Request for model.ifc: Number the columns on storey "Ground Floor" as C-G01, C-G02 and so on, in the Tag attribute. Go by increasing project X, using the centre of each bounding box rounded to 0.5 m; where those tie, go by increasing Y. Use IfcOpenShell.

First a look at what the model holds.

```python
import ifcopenshell
import ifcopenshell.util.element
import ifcopenshell.util.placement

model = ifcopenshell.open("model.ifc")
print(model.schema)
storey = next(s for s in model.by_type("IfcBuildingStorey") if s.Name == "Ground Floor")
columns = [e for e in ifcopenshell.util.element.get_decomposition(storey) if e.is_a("IfcColumn")]
for e in sorted(columns, key=lambda e: e.id()):
    origin = ifcopenshell.util.placement.get_local_placement(e.ObjectPlacement)[:3, 3]
    print(e.id(), e.Tag, e.Name, origin.round(2) + 0.0, sep=" | ")
```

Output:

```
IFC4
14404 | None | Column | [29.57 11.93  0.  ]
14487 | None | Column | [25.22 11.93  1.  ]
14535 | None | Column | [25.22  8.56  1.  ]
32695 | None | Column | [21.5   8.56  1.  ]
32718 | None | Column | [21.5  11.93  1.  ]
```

```python
import ifcopenshell
import ifcopenshell.geom
import ifcopenshell.util.element
import ifcopenshell.util.shape

model = ifcopenshell.open("model.ifc")
settings = ifcopenshell.geom.settings()
settings.set("use-world-coords", True)


def centre(element):
    shape = ifcopenshell.geom.create_shape(settings, element)
    return ifcopenshell.util.shape.get_bbox_centroid(shape.geometry)


storey = next(s for s in model.by_type("IfcBuildingStorey") if s.Name == "Ground Floor")
columns = [e for e in ifcopenshell.util.element.get_decomposition(storey) if e.is_a("IfcColumn")]

# Insertion points can sit at a corner or the storey origin, so sort by the geometry (in metres).
centres = {e: centre(e) for e in columns}
columns.sort(key=lambda e: (round(centres[e][0] / 0.5), centres[e][1]))

for i, e in enumerate(columns, start=1):
    number = f"C-G{i:02d}"
    e.Tag = number
    print(e.id(), number)

model.write("model_v2.ifc")
```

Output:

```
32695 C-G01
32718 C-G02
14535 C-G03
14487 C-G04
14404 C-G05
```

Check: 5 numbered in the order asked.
